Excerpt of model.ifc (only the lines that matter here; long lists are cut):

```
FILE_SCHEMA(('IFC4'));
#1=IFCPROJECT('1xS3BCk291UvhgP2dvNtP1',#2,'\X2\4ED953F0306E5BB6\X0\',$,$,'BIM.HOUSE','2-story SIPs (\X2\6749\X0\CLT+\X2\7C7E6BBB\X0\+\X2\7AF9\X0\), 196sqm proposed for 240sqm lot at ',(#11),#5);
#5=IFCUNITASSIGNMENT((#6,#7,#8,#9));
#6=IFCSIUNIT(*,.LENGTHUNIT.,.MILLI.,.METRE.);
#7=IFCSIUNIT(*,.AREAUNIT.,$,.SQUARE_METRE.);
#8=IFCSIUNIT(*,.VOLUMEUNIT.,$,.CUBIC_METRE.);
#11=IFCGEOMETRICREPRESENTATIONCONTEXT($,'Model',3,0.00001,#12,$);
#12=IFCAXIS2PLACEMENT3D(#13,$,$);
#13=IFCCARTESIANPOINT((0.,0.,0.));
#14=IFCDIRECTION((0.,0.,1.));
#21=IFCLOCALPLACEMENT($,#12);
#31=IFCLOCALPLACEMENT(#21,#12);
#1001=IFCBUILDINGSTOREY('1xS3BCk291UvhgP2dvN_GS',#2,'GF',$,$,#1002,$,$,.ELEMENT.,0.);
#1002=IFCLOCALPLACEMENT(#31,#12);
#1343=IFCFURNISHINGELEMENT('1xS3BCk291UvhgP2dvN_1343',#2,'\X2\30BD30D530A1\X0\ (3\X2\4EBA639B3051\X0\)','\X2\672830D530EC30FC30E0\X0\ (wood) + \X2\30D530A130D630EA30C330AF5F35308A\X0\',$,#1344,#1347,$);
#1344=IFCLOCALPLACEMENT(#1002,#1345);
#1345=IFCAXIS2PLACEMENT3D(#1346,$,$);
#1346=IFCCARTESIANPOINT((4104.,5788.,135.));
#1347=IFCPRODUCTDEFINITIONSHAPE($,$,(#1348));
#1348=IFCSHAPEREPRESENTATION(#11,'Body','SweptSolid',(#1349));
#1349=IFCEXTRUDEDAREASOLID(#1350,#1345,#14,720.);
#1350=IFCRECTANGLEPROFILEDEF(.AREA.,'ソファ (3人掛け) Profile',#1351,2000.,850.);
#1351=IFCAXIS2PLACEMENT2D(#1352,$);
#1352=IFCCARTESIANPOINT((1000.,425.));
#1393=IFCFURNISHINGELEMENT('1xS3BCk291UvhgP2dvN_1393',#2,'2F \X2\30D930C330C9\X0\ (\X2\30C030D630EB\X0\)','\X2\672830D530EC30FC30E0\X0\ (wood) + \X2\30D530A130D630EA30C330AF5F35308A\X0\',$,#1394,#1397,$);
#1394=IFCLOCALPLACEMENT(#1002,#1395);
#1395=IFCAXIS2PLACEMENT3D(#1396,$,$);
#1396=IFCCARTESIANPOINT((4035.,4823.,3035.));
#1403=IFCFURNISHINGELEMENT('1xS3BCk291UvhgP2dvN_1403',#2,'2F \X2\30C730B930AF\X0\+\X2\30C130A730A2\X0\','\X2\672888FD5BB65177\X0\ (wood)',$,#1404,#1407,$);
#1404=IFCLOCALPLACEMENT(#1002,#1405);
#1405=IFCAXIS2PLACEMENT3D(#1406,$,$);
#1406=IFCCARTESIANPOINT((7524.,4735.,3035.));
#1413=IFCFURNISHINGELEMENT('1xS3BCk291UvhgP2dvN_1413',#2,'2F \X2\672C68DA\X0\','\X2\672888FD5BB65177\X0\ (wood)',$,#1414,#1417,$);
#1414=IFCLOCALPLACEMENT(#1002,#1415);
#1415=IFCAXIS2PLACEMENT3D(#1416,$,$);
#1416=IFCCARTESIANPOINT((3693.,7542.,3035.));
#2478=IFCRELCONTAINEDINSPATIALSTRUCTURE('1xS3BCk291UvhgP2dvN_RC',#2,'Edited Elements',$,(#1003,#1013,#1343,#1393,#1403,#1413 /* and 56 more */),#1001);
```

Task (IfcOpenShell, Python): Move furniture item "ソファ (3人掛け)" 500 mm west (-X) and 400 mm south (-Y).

```python
import ifcopenshell
import ifcopenshell.api.geometry
import ifcopenshell.util.placement
import ifcopenshell.util.unit

model = ifcopenshell.open("model.ifc")
unit_scale = ifcopenshell.util.unit.calculate_unit_scale(model)

item = model.by_guid("1xS3BCk291UvhgP2dvN_1343")
matrix = ifcopenshell.util.placement.get_local_placement(item.ObjectPlacement)
matrix[0, 3] -= 0.5 / unit_scale
matrix[1, 3] -= 0.4 / unit_scale
ifcopenshell.api.geometry.edit_object_placement(model, product=item, matrix=matrix, is_si=False)

print(ifcopenshell.util.placement.get_local_placement(item.ObjectPlacement).round(3) + 0.0)

model.write("model_v2.ifc")
```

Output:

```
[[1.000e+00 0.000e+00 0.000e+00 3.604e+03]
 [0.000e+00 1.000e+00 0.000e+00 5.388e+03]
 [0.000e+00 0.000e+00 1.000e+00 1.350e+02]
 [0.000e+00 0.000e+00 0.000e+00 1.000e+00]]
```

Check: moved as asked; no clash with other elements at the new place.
